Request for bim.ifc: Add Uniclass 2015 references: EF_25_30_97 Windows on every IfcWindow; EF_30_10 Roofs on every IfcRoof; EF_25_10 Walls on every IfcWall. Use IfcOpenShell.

First a look at what the model holds.

```python
import ifcopenshell

model = ifcopenshell.open("bim.ifc")
print(model.schema)
print("classifications:", [c.Name for c in model.by_type("IfcClassification")])
for ifc_class in ("IfcDoor", "IfcRoof", "IfcStair", "IfcWall", "IfcWindow"):
    print(ifc_class, len(model.by_type(ifc_class)))
```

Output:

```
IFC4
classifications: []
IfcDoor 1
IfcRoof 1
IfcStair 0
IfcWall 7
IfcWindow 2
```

```python
import ifcopenshell
import ifcopenshell.api.classification

model = ifcopenshell.open("bim.ifc")

system = ifcopenshell.api.classification.add_classification(model, classification="Uniclass 2015")

codes = {
    "IfcWindow": ("EF_25_30_97", "Windows"),
    "IfcRoof": ("EF_30_10", "Roofs"),
    "IfcWall": ("EF_25_10", "Walls"),
}
for ifc_class, (code, name) in codes.items():
    products = model.by_type(ifc_class)
    ifcopenshell.api.classification.add_reference(
        model, products=products, classification=system, identification=code, name=name
    )
    print(code, len(products))

model.write("bim_edited.ifc")
```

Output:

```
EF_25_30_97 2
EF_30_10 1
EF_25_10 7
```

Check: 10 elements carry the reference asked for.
